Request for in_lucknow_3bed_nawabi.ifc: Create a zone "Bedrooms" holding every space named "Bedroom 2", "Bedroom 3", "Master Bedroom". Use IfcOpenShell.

First a look at what the model holds.

```python
import ifcopenshell

model = ifcopenshell.open("in_lucknow_3bed_nawabi.ifc")
print(model.schema)
seen = {}
for space in model.by_type("IfcSpace"):
    seen[space.LongName] = seen.get(space.LongName, 0) + 1
for name, count in sorted(seen.items(), key=str):
    print(count, "x", name)
print("zones:", [z.Name for z in model.by_type("IfcZone")][:20])
```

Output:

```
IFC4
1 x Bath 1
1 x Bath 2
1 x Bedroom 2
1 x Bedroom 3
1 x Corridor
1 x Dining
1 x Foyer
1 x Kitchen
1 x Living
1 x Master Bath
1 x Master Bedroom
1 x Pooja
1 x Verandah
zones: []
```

```python
import ifcopenshell
import ifcopenshell.api.group
import ifcopenshell.api.root

model = ifcopenshell.open("in_lucknow_3bed_nawabi.ifc")

names = {"Bedroom 2", "Bedroom 3", "Master Bedroom"}
spaces = [s for s in model.by_type("IfcSpace") if s.LongName in names]

zone = ifcopenshell.api.root.create_entity(model, ifc_class="IfcZone", name="Bedrooms")
ifcopenshell.api.group.assign_group(model, products=spaces, group=zone)
print(len(spaces), "spaces in", zone.Name)

model.write("in_lucknow_3bed_nawabi_rev.ifc")
```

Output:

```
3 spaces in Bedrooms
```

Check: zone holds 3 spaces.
